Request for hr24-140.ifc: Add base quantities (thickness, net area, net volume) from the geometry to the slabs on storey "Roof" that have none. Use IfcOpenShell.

First a look at what the model holds.

```python
import ifcopenshell
import ifcopenshell.util.element
import ifcopenshell.util.unit

model = ifcopenshell.open("hr24-140.ifc")
print(model.schema)
for unit_type in ("LENGTHUNIT", "AREAUNIT", "VOLUMEUNIT"):
    print(unit_type, ifcopenshell.util.unit.calculate_unit_scale(model, unit_type))
storey = next(s for s in model.by_type("IfcBuildingStorey") if s.Name == "Roof")
slabs = [e for e in ifcopenshell.util.element.get_decomposition(storey) if e.is_a("IfcSlab")]
for e in sorted(slabs, key=lambda e: e.id()):
    print(e.id(), e.is_a(), e.Name, list(ifcopenshell.util.element.get_psets(e, qtos_only=True)), sep=" | ")
```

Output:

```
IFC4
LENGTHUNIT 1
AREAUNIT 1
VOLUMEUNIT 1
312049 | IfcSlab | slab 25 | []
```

```python
import ifcopenshell
import ifcopenshell.api.pset
import ifcopenshell.geom
import ifcopenshell.util.element
import ifcopenshell.util.shape
import ifcopenshell.util.unit

model = ifcopenshell.open("hr24-140.ifc")
unit_scale = ifcopenshell.util.unit.calculate_unit_scale(model)
area_scale = ifcopenshell.util.unit.calculate_unit_scale(model, "AREAUNIT")
volume_scale = ifcopenshell.util.unit.calculate_unit_scale(model, "VOLUMEUNIT")
settings = ifcopenshell.geom.settings()

storey = next(s for s in model.by_type("IfcBuildingStorey") if s.Name == "Roof")
slabs = [e for e in ifcopenshell.util.element.get_decomposition(storey) if e.is_a("IfcSlab")]

for e in sorted(slabs, key=lambda e: e.id()):
    if ifcopenshell.util.element.get_psets(e, qtos_only=True, should_inherit=False):
        continue
    # Geometry comes back in metres, in the element's own axes.
    shape = ifcopenshell.geom.create_shape(settings, e)
    values = {
        "Width": ifcopenshell.util.shape.get_z(shape.geometry) / unit_scale,
        "NetArea": ifcopenshell.util.shape.get_footprint_area(shape.geometry) / area_scale,
        "NetVolume": ifcopenshell.util.shape.get_volume(shape.geometry) / volume_scale,
    }
    qto = ifcopenshell.api.pset.add_qto(model, product=e, name="Qto_SlabBaseQuantities")
    ifcopenshell.api.pset.edit_qto(model, qto=qto, properties=values)
    print(e.id(), {k: round(v, 3) for k, v in values.items()})

model.write("hr24-140_v2.ifc")
```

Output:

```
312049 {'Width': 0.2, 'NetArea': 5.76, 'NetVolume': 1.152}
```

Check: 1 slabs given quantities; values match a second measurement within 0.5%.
